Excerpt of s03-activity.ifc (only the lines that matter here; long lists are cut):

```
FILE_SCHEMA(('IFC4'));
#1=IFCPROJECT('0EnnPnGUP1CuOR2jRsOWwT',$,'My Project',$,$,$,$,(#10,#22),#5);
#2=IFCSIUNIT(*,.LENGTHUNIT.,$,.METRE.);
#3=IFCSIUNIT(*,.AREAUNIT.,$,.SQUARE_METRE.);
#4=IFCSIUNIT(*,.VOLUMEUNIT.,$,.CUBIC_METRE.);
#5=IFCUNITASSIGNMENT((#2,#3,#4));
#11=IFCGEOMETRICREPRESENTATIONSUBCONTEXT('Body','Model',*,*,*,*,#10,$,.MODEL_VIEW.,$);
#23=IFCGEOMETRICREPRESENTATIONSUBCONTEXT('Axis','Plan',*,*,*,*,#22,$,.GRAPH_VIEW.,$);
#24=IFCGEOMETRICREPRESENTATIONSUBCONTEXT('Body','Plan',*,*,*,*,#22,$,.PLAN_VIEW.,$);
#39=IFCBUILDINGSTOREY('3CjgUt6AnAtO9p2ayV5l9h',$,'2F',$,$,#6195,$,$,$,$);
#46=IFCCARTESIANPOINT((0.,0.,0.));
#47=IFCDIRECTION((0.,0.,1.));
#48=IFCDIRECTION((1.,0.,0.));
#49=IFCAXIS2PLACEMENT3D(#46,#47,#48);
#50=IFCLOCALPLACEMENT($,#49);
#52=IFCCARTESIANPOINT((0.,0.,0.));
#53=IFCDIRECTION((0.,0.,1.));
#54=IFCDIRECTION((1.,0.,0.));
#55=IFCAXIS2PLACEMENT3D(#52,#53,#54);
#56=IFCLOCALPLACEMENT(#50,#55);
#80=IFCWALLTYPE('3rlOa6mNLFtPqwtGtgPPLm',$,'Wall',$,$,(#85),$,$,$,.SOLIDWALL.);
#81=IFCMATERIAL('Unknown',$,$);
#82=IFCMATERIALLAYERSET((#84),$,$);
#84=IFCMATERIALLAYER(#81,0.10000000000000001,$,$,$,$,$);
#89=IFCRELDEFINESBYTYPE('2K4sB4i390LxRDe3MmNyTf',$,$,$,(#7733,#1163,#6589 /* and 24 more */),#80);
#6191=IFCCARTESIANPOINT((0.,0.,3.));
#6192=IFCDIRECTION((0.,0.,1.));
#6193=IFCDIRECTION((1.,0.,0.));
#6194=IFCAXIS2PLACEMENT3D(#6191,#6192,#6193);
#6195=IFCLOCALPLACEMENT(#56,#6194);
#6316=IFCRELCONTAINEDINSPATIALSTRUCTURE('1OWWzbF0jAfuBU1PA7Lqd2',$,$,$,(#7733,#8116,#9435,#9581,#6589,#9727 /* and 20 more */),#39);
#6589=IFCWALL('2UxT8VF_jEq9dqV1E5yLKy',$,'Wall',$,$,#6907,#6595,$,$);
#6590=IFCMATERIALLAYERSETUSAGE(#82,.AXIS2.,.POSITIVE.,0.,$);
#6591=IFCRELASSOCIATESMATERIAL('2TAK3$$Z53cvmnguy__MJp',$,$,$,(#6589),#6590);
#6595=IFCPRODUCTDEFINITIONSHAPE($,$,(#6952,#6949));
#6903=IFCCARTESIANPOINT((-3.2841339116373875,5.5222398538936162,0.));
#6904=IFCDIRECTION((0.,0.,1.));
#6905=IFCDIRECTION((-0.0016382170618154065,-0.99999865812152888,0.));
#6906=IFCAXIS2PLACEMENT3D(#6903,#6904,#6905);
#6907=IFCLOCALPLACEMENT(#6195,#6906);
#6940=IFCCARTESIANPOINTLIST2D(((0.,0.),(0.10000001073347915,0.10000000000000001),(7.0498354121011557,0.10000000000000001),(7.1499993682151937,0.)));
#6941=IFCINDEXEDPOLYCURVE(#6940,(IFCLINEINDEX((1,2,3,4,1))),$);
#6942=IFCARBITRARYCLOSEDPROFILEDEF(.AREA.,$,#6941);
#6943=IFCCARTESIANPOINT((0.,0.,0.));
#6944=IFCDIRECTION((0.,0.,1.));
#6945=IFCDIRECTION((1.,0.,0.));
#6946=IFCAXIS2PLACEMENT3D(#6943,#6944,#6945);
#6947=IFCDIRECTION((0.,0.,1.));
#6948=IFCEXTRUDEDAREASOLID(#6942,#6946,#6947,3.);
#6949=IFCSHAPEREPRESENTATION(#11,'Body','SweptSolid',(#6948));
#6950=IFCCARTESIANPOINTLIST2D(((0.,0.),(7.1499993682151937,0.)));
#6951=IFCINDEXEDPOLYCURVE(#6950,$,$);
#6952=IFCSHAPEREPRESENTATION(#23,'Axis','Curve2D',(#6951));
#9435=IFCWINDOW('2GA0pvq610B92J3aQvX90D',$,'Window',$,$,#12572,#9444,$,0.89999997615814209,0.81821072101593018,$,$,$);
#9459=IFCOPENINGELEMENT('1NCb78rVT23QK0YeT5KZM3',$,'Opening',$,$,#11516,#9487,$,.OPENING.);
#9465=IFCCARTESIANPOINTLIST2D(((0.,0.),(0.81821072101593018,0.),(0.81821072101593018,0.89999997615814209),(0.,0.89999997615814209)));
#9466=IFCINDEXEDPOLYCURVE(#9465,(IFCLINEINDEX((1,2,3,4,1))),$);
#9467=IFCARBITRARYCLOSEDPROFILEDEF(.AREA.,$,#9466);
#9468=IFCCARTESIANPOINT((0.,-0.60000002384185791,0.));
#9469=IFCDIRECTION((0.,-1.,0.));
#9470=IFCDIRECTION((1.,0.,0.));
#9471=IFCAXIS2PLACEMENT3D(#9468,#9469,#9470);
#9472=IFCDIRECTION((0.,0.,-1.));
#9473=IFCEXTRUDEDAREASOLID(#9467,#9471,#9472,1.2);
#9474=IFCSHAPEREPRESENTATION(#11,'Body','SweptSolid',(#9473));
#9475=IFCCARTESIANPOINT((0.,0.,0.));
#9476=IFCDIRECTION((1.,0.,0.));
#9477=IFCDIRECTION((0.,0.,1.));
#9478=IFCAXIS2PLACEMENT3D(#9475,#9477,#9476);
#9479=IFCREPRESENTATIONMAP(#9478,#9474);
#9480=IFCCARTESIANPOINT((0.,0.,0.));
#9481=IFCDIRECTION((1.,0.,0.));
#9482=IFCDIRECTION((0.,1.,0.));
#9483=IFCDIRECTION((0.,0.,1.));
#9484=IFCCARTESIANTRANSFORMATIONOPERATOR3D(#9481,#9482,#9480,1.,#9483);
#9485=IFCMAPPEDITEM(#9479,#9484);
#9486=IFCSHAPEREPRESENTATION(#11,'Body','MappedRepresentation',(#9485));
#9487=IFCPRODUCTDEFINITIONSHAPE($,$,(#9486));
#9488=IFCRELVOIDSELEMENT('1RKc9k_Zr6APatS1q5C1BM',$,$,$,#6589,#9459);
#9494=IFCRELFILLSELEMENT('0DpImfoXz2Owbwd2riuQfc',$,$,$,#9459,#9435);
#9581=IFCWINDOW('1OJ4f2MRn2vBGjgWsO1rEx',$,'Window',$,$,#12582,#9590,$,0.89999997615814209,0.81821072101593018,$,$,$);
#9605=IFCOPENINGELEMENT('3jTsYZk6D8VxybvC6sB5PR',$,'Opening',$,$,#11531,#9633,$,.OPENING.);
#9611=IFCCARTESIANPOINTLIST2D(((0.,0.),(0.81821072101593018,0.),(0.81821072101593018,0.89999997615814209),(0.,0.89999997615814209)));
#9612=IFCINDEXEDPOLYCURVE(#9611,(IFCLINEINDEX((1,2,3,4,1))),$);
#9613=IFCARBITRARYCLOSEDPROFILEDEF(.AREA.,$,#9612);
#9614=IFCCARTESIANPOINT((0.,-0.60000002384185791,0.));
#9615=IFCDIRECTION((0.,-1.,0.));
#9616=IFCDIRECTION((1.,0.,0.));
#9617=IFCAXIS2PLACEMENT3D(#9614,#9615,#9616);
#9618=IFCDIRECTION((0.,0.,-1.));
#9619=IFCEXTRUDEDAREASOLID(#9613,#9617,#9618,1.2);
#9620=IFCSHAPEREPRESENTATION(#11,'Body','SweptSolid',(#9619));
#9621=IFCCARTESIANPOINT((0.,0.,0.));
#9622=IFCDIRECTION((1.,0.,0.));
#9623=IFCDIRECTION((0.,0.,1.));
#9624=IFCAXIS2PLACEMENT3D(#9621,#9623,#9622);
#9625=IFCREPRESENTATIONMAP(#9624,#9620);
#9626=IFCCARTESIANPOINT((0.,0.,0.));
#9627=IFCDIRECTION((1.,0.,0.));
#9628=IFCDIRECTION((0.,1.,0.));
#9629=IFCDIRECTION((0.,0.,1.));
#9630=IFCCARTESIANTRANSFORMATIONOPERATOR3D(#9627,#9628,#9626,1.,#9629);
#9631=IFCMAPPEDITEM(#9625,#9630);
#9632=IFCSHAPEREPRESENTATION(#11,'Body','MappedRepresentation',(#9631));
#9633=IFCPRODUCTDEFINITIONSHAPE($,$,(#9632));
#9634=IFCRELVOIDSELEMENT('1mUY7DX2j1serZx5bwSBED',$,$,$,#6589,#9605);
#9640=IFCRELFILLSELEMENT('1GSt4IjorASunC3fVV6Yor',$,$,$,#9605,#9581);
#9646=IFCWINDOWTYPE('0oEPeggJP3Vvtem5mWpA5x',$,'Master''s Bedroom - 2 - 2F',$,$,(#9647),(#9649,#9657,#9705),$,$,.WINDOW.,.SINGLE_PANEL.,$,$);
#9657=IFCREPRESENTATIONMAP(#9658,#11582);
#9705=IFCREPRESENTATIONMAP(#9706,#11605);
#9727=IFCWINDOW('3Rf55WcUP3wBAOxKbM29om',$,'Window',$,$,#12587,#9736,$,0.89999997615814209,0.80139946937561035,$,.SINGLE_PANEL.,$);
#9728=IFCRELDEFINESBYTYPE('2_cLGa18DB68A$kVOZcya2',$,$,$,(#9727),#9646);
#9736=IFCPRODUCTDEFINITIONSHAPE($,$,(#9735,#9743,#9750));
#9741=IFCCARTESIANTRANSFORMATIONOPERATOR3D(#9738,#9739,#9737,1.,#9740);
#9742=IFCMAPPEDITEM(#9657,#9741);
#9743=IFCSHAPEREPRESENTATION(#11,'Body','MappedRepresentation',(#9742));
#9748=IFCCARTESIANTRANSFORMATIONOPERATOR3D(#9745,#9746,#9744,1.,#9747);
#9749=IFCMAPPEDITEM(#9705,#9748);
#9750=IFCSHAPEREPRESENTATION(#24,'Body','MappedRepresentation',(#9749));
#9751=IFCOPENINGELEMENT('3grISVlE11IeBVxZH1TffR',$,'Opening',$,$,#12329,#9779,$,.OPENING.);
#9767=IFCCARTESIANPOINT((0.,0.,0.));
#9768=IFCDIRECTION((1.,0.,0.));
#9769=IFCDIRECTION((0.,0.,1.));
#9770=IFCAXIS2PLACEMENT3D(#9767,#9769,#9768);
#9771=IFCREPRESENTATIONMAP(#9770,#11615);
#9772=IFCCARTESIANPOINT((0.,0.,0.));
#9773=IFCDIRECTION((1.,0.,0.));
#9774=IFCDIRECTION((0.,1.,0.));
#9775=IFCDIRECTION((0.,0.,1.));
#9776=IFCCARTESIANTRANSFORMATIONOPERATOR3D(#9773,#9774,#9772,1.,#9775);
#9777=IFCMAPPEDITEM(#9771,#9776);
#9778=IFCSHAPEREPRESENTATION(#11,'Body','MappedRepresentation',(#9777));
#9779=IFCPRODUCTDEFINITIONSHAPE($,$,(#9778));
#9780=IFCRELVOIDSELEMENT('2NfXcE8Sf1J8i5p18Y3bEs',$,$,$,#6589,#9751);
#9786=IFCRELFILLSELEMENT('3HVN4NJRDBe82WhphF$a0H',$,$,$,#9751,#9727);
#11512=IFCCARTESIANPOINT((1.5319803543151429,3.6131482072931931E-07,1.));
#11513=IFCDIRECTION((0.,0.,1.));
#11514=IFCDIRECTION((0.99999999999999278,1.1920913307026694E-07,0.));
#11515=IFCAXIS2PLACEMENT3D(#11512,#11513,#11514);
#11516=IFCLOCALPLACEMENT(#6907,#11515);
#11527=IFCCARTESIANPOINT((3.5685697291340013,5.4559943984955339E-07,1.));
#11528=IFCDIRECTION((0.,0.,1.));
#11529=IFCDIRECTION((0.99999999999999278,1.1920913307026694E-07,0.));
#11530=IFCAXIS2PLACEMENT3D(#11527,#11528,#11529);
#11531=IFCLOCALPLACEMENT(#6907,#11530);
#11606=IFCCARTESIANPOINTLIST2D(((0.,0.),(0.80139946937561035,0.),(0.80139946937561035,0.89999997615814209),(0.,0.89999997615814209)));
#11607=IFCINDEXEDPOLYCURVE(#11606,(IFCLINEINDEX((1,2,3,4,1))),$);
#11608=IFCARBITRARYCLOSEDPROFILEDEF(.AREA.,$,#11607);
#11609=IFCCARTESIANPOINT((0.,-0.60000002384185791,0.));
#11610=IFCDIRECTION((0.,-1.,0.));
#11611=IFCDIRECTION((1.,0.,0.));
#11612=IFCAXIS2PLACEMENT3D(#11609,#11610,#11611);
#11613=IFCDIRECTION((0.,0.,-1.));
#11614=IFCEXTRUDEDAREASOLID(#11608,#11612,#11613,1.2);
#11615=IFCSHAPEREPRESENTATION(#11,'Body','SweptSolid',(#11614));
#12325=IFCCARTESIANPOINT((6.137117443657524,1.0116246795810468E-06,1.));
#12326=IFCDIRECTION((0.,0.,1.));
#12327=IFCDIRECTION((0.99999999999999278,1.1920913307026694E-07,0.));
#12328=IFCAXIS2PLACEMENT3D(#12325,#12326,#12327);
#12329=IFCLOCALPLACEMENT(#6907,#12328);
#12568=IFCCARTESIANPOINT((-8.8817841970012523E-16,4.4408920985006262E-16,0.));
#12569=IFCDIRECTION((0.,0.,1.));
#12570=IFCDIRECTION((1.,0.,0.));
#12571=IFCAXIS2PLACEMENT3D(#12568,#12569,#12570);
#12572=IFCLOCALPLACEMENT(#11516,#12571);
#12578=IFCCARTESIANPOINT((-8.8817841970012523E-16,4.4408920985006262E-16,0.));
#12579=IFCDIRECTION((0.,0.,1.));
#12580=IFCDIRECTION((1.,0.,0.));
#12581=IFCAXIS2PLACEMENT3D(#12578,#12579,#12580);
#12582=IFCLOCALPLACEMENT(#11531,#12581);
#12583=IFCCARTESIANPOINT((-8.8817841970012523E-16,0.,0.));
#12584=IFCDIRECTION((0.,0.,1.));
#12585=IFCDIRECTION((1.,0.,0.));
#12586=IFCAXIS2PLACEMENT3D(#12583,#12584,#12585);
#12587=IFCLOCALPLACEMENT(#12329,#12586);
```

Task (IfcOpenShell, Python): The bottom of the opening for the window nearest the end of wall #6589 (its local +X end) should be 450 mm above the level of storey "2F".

```python
import numpy as np
import ifcopenshell
import ifcopenshell.api.geometry
import ifcopenshell.geom
import ifcopenshell.util.element
import ifcopenshell.util.placement
import ifcopenshell.util.shape
import ifcopenshell.util.unit

model = ifcopenshell.open("s03-activity.ifc")
unit_scale = ifcopenshell.util.unit.calculate_unit_scale(model)

window = model.by_guid("3Rf55WcUP3wBAOxKbM29om")
opening = window.FillsVoids[0].RelatingOpeningElement
storey = ifcopenshell.util.element.get_container(window, ifc_class="IfcBuildingStorey")
level = ifcopenshell.util.placement.get_local_placement(storey.ObjectPlacement)[2, 3]

# The opening's origin need not be at the sill, so measure its lowest point.
shape = ifcopenshell.geom.create_shape(ifcopenshell.geom.settings(), opening)
bottom = ifcopenshell.util.shape.get_shape_bottom_elevation(shape, shape.geometry) / unit_scale
dz = level + 0.45 / unit_scale - bottom

shift = np.array([0.0, 0.0, dz])
# The window is placed relative to its opening, so it follows when the opening moves.
matrix = ifcopenshell.util.placement.get_local_placement(opening.ObjectPlacement)
matrix[:3, 3] += shift
ifcopenshell.api.geometry.edit_object_placement(
    model, product=opening, matrix=matrix, is_si=False, should_transform_children=True
)

print(f"moved by {dz * unit_scale:+.3f} m")

model.write("s03-activity-out.ifc")
```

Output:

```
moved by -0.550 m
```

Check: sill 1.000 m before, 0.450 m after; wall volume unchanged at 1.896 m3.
